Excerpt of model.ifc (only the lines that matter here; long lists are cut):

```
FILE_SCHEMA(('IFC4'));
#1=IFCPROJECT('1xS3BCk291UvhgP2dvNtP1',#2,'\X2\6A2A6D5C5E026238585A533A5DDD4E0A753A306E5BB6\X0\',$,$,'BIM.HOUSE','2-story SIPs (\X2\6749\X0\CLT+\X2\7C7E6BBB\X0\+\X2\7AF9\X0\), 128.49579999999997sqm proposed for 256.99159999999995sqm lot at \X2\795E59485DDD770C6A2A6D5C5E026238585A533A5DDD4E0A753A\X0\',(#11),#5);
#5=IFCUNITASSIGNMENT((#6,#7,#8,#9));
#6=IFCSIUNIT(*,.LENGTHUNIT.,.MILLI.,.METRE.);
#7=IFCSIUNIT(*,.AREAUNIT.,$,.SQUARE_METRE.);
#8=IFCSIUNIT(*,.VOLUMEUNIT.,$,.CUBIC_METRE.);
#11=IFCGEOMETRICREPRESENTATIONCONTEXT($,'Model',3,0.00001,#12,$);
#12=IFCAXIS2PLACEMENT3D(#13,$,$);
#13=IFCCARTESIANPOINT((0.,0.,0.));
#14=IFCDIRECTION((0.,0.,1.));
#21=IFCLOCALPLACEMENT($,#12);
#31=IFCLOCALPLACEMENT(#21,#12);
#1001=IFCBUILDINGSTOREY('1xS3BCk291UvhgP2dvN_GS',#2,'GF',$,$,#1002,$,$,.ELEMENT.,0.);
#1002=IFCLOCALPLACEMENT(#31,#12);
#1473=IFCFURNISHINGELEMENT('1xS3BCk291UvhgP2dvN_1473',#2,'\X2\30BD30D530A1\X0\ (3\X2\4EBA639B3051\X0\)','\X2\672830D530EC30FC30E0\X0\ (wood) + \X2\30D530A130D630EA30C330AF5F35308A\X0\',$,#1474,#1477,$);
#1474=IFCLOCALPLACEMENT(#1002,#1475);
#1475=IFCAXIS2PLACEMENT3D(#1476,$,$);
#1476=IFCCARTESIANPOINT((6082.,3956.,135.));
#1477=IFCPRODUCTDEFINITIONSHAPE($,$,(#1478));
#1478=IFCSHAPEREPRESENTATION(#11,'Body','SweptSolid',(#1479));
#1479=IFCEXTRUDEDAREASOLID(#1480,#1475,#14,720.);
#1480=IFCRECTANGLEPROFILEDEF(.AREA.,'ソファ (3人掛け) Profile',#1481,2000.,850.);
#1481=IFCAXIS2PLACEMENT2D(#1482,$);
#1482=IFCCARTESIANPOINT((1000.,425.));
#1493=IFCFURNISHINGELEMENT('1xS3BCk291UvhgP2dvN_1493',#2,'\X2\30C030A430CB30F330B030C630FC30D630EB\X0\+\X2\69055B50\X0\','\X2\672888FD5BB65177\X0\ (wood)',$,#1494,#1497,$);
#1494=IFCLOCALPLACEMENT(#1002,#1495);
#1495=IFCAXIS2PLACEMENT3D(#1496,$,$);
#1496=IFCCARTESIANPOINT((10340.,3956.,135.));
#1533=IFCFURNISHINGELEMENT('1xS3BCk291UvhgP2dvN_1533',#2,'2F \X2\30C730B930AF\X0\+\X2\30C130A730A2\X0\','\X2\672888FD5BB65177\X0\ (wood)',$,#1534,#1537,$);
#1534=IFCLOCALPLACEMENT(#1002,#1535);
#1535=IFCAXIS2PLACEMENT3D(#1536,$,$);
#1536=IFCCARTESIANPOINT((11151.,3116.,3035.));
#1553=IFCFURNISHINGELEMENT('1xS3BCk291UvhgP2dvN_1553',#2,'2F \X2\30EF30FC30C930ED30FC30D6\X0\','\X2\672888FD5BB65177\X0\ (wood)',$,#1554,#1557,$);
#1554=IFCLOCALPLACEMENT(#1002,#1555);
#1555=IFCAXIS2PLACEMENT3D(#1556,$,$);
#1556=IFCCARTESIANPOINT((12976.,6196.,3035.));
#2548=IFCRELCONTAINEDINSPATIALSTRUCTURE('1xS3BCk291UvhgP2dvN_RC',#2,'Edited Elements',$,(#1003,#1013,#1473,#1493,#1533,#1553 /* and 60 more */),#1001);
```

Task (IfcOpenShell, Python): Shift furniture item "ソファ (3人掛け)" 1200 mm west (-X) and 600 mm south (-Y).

```python
import ifcopenshell
import ifcopenshell.api.geometry
import ifcopenshell.util.placement
import ifcopenshell.util.unit

model = ifcopenshell.open("model.ifc")
unit_scale = ifcopenshell.util.unit.calculate_unit_scale(model)

item = model.by_id(1473)
matrix = ifcopenshell.util.placement.get_local_placement(item.ObjectPlacement)
matrix[0, 3] -= 1.2 / unit_scale
matrix[1, 3] -= 0.6 / unit_scale
ifcopenshell.api.geometry.edit_object_placement(model, product=item, matrix=matrix, is_si=False)

print(ifcopenshell.util.placement.get_local_placement(item.ObjectPlacement).round(3) + 0.0)

model.write("model_updated.ifc")
```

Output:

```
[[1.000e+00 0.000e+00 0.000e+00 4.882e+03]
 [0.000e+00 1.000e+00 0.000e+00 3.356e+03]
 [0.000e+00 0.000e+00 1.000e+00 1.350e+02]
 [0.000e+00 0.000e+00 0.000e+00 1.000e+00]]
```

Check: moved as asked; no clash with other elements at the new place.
